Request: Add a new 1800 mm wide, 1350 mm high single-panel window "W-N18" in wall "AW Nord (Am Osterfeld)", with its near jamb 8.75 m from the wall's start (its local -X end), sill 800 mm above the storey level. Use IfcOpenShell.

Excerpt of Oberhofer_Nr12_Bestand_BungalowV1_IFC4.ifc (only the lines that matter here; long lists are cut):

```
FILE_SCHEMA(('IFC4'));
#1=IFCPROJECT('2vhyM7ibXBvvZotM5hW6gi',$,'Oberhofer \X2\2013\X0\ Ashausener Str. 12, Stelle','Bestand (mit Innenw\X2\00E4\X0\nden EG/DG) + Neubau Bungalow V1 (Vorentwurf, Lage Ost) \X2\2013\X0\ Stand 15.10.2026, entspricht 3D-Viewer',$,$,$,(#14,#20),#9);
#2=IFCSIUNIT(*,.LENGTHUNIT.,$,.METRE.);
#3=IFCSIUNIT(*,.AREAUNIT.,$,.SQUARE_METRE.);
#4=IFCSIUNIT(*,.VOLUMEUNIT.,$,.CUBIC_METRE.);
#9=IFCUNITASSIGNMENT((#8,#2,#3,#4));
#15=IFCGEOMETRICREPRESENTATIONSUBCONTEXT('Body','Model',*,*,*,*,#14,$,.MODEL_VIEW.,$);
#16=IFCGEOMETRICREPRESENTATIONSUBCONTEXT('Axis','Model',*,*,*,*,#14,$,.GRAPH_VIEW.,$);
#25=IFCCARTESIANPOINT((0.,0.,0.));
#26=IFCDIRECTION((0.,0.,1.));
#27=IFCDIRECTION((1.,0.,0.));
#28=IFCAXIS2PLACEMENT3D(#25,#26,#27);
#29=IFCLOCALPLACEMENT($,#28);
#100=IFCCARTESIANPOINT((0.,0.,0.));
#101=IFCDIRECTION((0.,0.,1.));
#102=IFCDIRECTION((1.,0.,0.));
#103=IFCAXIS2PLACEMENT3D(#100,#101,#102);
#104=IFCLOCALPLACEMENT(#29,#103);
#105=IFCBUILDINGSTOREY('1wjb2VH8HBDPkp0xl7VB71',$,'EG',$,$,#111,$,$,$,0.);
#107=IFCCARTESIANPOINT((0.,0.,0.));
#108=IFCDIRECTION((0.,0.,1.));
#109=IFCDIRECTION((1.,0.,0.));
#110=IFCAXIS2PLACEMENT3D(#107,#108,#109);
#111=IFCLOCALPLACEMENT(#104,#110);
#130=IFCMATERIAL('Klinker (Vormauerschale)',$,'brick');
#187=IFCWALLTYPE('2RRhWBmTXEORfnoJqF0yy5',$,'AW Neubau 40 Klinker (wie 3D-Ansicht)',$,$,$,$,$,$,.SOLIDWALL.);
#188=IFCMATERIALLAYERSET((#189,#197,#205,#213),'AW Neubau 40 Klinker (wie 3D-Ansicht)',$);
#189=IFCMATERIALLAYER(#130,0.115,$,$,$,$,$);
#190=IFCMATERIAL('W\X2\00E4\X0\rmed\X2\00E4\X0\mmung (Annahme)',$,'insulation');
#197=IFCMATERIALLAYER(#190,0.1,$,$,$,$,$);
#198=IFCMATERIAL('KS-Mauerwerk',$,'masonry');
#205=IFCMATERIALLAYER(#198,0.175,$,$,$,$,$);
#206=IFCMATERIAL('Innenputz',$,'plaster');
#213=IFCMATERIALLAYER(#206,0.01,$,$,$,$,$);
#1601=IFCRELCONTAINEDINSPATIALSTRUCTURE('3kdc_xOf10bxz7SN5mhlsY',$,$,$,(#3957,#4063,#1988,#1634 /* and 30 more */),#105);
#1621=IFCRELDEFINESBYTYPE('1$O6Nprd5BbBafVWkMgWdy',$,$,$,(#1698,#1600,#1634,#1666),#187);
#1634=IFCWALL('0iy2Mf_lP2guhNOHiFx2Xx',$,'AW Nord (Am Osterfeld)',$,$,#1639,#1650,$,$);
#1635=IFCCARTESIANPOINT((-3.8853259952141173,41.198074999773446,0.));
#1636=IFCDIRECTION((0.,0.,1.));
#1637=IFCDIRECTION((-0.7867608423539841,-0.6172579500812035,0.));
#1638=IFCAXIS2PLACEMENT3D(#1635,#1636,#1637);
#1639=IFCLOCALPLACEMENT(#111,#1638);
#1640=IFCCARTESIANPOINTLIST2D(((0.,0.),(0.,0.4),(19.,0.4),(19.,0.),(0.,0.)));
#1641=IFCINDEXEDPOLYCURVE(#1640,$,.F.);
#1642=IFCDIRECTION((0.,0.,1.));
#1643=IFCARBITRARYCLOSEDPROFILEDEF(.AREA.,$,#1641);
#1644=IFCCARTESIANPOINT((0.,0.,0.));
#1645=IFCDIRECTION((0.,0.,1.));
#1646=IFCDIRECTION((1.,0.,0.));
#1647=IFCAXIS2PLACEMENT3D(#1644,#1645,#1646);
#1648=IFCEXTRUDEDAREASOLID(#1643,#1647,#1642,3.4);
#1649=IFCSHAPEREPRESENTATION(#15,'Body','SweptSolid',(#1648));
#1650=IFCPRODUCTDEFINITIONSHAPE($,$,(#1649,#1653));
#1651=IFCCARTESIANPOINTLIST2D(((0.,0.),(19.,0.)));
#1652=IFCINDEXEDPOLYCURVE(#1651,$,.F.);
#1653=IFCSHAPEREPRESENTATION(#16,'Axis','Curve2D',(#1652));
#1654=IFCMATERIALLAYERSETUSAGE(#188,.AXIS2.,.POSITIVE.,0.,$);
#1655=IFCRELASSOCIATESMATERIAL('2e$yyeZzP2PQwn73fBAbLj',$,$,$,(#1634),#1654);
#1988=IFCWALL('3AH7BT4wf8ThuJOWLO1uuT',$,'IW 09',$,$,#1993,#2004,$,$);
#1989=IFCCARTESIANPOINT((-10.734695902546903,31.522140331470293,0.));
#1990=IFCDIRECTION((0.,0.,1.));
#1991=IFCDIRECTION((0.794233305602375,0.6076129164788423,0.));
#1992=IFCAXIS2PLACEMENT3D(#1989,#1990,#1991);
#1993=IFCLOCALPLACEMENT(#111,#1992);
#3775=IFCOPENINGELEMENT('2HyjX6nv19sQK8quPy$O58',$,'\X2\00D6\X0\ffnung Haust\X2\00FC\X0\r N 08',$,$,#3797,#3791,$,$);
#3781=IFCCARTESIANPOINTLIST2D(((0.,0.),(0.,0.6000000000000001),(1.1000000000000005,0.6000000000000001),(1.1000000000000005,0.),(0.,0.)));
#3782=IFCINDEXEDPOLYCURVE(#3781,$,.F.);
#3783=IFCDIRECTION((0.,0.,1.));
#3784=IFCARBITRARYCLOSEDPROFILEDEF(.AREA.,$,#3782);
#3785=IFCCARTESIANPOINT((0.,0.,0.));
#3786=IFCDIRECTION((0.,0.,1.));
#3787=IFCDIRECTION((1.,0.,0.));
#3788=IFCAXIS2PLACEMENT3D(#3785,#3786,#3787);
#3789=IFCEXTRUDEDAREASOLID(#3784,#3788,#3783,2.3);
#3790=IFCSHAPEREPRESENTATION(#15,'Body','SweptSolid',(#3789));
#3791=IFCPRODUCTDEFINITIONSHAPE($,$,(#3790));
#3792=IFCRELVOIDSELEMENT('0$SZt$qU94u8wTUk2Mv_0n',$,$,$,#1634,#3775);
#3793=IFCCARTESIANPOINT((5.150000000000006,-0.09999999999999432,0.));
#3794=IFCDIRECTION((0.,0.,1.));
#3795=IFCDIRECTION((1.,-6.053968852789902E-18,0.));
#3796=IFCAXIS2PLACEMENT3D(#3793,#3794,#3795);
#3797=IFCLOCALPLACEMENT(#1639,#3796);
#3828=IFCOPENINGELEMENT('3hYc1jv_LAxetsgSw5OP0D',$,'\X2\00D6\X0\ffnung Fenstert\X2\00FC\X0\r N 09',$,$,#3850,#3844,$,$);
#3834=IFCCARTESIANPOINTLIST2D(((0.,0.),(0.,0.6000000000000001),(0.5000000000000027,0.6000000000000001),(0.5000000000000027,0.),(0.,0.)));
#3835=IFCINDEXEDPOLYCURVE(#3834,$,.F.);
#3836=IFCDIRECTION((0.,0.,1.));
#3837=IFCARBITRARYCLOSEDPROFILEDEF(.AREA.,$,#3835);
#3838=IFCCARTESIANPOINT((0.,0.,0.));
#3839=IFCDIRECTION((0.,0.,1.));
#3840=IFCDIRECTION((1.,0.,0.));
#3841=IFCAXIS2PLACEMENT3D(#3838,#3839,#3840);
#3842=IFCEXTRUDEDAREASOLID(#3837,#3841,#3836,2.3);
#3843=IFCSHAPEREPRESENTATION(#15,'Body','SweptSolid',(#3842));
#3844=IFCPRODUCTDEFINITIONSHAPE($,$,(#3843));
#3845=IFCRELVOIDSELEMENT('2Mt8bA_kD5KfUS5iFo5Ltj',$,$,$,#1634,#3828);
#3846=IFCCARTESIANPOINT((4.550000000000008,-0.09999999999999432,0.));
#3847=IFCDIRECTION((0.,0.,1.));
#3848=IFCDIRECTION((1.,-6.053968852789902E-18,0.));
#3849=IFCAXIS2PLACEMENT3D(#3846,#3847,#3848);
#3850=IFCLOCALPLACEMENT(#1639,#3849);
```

```python
import numpy as np
import ifcopenshell
import ifcopenshell.api.feature
import ifcopenshell.api.geometry
import ifcopenshell.api.root
import ifcopenshell.api.spatial
import ifcopenshell.geom
import ifcopenshell.util.element
import ifcopenshell.util.placement
import ifcopenshell.util.representation
import ifcopenshell.util.shape
import ifcopenshell.util.unit

model = ifcopenshell.open("Oberhofer_Nr12_Bestand_BungalowV1_IFC4.ifc")
unit_scale = ifcopenshell.util.unit.calculate_unit_scale(model)
settings = ifcopenshell.geom.settings()


def volume(element):
    """Net volume in cubic metres, openings subtracted."""
    shape = ifcopenshell.geom.create_shape(settings, element)
    return ifcopenshell.util.shape.get_volume(shape.geometry)


wall = model.by_guid("0iy2Mf_lP2guhNOHiFx2Xx")
storey = ifcopenshell.util.element.get_container(wall, ifc_class="IfcBuildingStorey")
context = ifcopenshell.util.representation.get_context(model, "Model", "Body", "MODEL_VIEW")
before = volume(wall)

width, height, from_end, sill = 1.8, 1.35, 8.75, 0.8  # metres

# The wall runs along its own X axis, and the end named is its -X end.
wall_shape = ifcopenshell.geom.create_shape(settings, wall)
x, y, z = ifcopenshell.util.shape.get_vertices(wall_shape.geometry).T
start = x.min() + from_end
face, thickness = float(y.min()), float(y.max() - y.min())
wall_matrix = ifcopenshell.util.placement.get_local_placement(wall.ObjectPlacement)
level = ifcopenshell.util.placement.get_local_placement(storey.ObjectPlacement)[2, 3]


def in_wall(x, y):
    """Placement at x, y metres in the wall's axes, at sill height."""
    matrix = wall_matrix.copy()
    matrix[:, 3] = wall_matrix @ np.array([x / unit_scale, y / unit_scale, 0.0, 1.0])
    matrix[2, 3] = level + sill / unit_scale
    return matrix


# Opening: a box that overshoots both wall faces by 50 mm.
opening = ifcopenshell.api.root.create_entity(model, ifc_class="IfcOpeningElement", predefined_type="OPENING")
box = ifcopenshell.api.geometry.add_wall_representation(
    model, context=context, length=width, height=height, thickness=thickness + 0.1
)
ifcopenshell.api.geometry.assign_representation(model, product=opening, representation=box)
ifcopenshell.api.geometry.edit_object_placement(model, product=opening, matrix=in_wall(start, face - 0.05), is_si=False)
ifcopenshell.api.feature.add_feature(model, feature=opening, element=wall)

window = ifcopenshell.api.root.create_entity(model, ifc_class="IfcWindow", name="W-N18", predefined_type="WINDOW")
window.OverallWidth, window.OverallHeight = width / unit_scale, height / unit_scale
window.PartitioningType = "SINGLE_PANEL"
body = ifcopenshell.api.geometry.add_window_representation(
    model,
    context=context,
    overall_width=window.OverallWidth,
    overall_height=window.OverallHeight,
    partition_type="SINGLE_PANEL",
)
ifcopenshell.api.geometry.assign_representation(model, product=window, representation=body)
ifcopenshell.api.spatial.assign_container(model, products=[window], relating_structure=storey)
ifcopenshell.api.feature.add_filling(model, opening=opening, element=window)

# Centre the window in the wall's thickness.
ifcopenshell.api.geometry.edit_object_placement(model, product=window, matrix=in_wall(start, face), is_si=False)
window_shape = ifcopenshell.geom.create_shape(settings, window)
depth = ifcopenshell.util.shape.get_vertices(window_shape.geometry)[:, 1]
offset = face + thickness / 2 - (depth.min() + depth.max()) / 2
ifcopenshell.api.geometry.edit_object_placement(model, product=window, matrix=in_wall(start, offset), is_si=False)

after = volume(wall)

print(f"wall volume {before:.3f} -> {after:.3f} m3")

model.write("Oberhofer_Nr12_Bestand_BungalowV1_IFC4_edited.ifc")
```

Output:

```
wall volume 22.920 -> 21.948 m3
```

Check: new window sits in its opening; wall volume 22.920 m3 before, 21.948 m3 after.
